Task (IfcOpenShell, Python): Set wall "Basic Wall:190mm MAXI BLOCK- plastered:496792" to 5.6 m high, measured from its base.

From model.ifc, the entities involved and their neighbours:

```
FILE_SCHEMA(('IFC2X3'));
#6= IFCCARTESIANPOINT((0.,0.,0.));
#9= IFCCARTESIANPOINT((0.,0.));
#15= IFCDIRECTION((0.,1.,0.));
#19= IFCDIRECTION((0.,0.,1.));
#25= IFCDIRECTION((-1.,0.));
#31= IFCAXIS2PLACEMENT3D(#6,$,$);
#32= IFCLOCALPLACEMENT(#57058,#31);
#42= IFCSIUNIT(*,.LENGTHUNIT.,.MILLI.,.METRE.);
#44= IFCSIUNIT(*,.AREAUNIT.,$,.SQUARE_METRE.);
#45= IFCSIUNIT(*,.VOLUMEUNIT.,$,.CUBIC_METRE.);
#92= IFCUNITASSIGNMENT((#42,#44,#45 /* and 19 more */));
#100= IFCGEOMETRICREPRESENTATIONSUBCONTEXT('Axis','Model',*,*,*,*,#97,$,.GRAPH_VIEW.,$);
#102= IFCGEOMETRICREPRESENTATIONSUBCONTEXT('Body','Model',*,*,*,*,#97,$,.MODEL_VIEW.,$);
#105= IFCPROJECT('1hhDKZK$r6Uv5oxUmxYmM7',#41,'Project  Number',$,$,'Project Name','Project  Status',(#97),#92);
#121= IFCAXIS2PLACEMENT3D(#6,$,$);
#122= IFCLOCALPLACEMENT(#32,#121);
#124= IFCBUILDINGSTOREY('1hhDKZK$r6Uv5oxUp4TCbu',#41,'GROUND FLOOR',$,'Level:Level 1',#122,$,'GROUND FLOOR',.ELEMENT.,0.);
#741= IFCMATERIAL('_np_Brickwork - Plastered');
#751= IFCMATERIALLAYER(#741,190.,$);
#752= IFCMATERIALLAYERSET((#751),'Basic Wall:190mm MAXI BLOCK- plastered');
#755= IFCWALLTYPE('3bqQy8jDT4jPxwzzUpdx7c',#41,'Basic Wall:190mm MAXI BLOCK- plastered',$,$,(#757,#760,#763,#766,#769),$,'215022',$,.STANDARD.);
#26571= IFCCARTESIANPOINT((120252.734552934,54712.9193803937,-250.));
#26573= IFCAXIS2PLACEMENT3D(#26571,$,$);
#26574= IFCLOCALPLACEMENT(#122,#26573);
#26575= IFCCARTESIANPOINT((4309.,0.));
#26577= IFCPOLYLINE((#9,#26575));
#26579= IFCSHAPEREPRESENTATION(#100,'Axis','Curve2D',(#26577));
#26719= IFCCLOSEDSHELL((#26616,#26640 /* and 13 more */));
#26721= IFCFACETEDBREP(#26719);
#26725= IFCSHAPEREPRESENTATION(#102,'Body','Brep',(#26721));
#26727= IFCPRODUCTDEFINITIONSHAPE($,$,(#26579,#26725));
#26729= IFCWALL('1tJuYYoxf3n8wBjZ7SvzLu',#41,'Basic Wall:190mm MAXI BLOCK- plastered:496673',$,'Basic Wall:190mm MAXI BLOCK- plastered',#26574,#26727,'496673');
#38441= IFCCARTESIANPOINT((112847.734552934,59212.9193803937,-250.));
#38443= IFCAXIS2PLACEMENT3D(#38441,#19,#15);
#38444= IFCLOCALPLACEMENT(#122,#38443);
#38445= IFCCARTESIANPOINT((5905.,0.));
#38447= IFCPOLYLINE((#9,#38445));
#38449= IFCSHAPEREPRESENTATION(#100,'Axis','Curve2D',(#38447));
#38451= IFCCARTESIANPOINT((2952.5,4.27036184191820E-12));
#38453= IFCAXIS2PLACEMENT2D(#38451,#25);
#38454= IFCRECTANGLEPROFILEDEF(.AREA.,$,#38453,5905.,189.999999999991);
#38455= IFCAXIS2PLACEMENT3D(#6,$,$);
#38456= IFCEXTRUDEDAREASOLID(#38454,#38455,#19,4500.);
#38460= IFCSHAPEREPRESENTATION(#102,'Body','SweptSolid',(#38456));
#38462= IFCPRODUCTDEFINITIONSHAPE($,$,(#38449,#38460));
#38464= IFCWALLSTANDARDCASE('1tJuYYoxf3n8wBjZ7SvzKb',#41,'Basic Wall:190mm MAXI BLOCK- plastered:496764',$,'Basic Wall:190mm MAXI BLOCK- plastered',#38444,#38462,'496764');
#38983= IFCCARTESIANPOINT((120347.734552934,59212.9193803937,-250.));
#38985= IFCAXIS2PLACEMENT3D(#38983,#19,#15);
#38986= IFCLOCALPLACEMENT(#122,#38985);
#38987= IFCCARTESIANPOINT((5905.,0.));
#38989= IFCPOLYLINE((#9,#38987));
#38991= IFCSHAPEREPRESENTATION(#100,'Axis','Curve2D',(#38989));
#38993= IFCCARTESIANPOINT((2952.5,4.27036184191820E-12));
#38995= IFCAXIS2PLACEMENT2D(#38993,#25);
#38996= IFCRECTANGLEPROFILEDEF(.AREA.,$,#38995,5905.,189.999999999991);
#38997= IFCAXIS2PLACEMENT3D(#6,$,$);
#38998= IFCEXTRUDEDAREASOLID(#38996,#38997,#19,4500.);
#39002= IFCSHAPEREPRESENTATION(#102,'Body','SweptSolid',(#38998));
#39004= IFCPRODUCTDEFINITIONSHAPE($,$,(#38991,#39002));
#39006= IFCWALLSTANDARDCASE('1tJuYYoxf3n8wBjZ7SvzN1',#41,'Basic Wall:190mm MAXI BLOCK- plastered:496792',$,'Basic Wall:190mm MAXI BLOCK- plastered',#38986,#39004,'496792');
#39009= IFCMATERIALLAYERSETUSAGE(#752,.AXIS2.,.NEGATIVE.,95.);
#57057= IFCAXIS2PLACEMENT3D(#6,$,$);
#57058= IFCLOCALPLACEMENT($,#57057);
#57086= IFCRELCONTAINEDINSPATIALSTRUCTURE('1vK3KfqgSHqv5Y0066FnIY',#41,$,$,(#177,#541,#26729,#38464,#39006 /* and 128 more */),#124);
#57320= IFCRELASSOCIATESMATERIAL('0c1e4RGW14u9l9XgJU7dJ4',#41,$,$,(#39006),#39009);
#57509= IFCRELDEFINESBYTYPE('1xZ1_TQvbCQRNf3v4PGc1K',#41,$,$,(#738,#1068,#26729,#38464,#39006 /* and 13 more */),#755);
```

```python
import ifcopenshell
import ifcopenshell.geom
import ifcopenshell.util.representation
import ifcopenshell.util.shape

model = ifcopenshell.open("model.ifc")
settings = ifcopenshell.geom.settings()


def volume(element):
    """Net volume in cubic metres, openings subtracted."""
    shape = ifcopenshell.geom.create_shape(settings, element)
    return ifcopenshell.util.shape.get_volume(shape.geometry)


wall = model.by_guid("1tJuYYoxf3n8wBjZ7SvzN1")
before = volume(wall)

body = ifcopenshell.util.representation.get_representation(wall, "Model", "Body")
solid = body.Items[0]
old_height = solid.Depth
solid.Depth = 5600.0
after = volume(wall)

print(f"height {old_height:g} -> {solid.Depth:g}, volume {before:.3f} -> {after:.3f} m3")

model.write("model-out.ifc")
```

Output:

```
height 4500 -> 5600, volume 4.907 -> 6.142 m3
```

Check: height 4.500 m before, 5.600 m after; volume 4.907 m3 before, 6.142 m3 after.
